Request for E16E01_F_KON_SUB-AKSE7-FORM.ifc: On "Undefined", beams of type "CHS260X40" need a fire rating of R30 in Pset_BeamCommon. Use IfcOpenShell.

First a look at what the model holds.

```python
import ifcopenshell
import ifcopenshell.util.element

model = ifcopenshell.open("E16E01_F_KON_SUB-AKSE7-FORM.ifc")
print(model.schema)
storey = next(s for s in model.by_type("IfcBuildingStorey") if s.Name == "Undefined")
beams = [e for e in ifcopenshell.util.element.get_decomposition(storey) if e.is_a("IfcBeam")]
seen = {}
for e in beams:
    element_type = ifcopenshell.util.element.get_type(e)
    key = (element_type.Name if element_type != e and element_type else None, ifcopenshell.util.element.get_pset(e, "Pset_BeamCommon", "FireRating"))
    seen[key] = seen.get(key, 0) + 1
for (name, value), count in sorted(seen.items(), key=str):
    print(count, "x", name, "|", value)
```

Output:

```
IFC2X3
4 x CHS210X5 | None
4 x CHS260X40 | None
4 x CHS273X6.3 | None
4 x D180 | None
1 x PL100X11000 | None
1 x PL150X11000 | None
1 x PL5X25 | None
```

```python
import ifcopenshell
import ifcopenshell.api.pset
import ifcopenshell.util.element

model = ifcopenshell.open("E16E01_F_KON_SUB-AKSE7-FORM.ifc")

storey = next(s for s in model.by_type("IfcBuildingStorey") if s.Name == "Undefined")
beams = [e for e in ifcopenshell.util.element.get_decomposition(storey) if e.is_a("IfcBeam")]

count = 0
for e in beams:
    element_type = ifcopenshell.util.element.get_type(e)
    if element_type in (None, e) or element_type.Name != "CHS260X40":
        continue
    found = ifcopenshell.util.element.get_pset(e, "Pset_BeamCommon", should_inherit=False)
    if found:
        pset = model.by_id(found["id"])
        if len(ifcopenshell.util.element.get_elements_by_pset(pset)) > 1:
            pset = ifcopenshell.api.pset.unshare_pset(model, products=[e], pset=pset)[0]
    else:
        pset = ifcopenshell.api.pset.add_pset(model, product=e, name="Pset_BeamCommon")
    ifcopenshell.api.pset.edit_pset(model, pset=pset, properties={"FireRating": "R30"})
    count += 1

print(count, "beams updated")

model.write("E16E01_F_KON_SUB-AKSE7-FORM_updated.ifc")
```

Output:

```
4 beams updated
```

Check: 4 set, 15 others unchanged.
